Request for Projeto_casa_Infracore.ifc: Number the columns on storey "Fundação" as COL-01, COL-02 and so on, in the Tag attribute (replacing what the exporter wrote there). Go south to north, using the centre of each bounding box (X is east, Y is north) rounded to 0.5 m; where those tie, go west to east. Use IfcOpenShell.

First a look at what the model holds.

```python
import ifcopenshell
import ifcopenshell.util.element
import ifcopenshell.util.placement

model = ifcopenshell.open("Projeto_casa_Infracore.ifc")
print(model.schema)
storey = next(s for s in model.by_type("IfcBuildingStorey") if s.Name == "Fundação")
columns = [e for e in ifcopenshell.util.element.get_decomposition(storey) if e.is_a("IfcColumn")]
for e in sorted(columns, key=lambda e: e.id()):
    origin = ifcopenshell.util.placement.get_local_placement(e.ObjectPlacement)[:3, 3]
    print(e.id(), e.Tag, e.Name, origin.round(2) + 0.0, sep=" | ")
```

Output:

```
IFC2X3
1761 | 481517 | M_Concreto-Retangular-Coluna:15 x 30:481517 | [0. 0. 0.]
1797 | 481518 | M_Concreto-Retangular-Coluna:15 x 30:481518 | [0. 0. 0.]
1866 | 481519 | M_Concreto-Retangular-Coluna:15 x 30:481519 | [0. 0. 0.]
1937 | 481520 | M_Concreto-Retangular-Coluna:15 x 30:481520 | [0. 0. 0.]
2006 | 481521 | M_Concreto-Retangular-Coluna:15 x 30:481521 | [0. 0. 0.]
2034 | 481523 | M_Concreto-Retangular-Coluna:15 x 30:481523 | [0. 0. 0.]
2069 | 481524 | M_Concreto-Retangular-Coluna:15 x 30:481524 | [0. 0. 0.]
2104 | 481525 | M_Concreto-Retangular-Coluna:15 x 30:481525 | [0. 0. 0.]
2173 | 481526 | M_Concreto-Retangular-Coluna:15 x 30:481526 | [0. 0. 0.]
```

```python
import ifcopenshell
import ifcopenshell.geom
import ifcopenshell.util.element
import ifcopenshell.util.shape

model = ifcopenshell.open("Projeto_casa_Infracore.ifc")
settings = ifcopenshell.geom.settings()
settings.set("use-world-coords", True)


def centre(element):
    shape = ifcopenshell.geom.create_shape(settings, element)
    return ifcopenshell.util.shape.get_bbox_centroid(shape.geometry)


storey = next(s for s in model.by_type("IfcBuildingStorey") if s.Name == "Fundação")
columns = [e for e in ifcopenshell.util.element.get_decomposition(storey) if e.is_a("IfcColumn")]

# Insertion points can sit at a corner or the storey origin, so sort by the geometry (in metres).
centres = {e: centre(e) for e in columns}
columns.sort(key=lambda e: (round(centres[e][1] / 0.5), centres[e][0]))

for i, e in enumerate(columns, start=1):
    number = f"COL-{i:02d}"
    e.Tag = number
    print(e.id(), number)

model.write("Projeto_casa_Infracore_updated.ifc")
```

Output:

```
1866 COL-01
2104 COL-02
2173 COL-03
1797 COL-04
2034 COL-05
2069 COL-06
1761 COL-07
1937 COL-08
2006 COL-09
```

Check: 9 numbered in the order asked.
